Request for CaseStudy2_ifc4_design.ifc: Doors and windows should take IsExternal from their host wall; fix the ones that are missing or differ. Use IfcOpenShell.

First a look at what the model holds.

```python
import ifcopenshell
import ifcopenshell.util.element

model = ifcopenshell.open("CaseStudy2_ifc4_design.ifc")
print(model.schema)
seen = {}
for e in model.by_type("IfcDoor") + model.by_type("IfcWindow"):
    if not e.FillsVoids:
        continue
    host = e.FillsVoids[0].RelatingOpeningElement.VoidsElements[0].RelatingBuildingElement
    own = ifcopenshell.util.element.get_pset(e, f"Pset_{e.is_a()[3:].removesuffix('StandardCase')}Common", "IsExternal")
    wall = ifcopenshell.util.element.get_pset(host, "Pset_WallCommon", "IsExternal")
    seen[e.is_a(), own, wall] = seen.get((e.is_a(), own, wall), 0) + 1
for (cls, own, wall), count in sorted(seen.items(), key=str):
    print(count, cls, "IsExternal:", own, "| host wall:", wall)
```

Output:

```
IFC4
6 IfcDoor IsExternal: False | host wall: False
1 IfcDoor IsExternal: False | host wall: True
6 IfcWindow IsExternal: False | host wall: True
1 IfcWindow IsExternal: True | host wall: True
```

```python
import ifcopenshell
import ifcopenshell.api.pset
import ifcopenshell.util.element

model = ifcopenshell.open("CaseStudy2_ifc4_design.ifc")

count = 0
for ifc_class, pset_name in (("IfcDoor", "Pset_DoorCommon"), ("IfcWindow", "Pset_WindowCommon")):
    for e in model.by_type(ifc_class):
        if not e.FillsVoids:
            continue
        host = e.FillsVoids[0].RelatingOpeningElement.VoidsElements[0].RelatingBuildingElement
        external = ifcopenshell.util.element.get_pset(host, "Pset_WallCommon", "IsExternal")
        if external is None or ifcopenshell.util.element.get_pset(e, pset_name, "IsExternal") == external:
            continue
        pset = ifcopenshell.api.pset.add_pset(model, product=e, name=pset_name)
        ifcopenshell.api.pset.edit_pset(model, pset=pset, properties={"IsExternal": external})
        count += 1

print(count, "updated")

model.write("CaseStudy2_ifc4_design-out.ifc")
```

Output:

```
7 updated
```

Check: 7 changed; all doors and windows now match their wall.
